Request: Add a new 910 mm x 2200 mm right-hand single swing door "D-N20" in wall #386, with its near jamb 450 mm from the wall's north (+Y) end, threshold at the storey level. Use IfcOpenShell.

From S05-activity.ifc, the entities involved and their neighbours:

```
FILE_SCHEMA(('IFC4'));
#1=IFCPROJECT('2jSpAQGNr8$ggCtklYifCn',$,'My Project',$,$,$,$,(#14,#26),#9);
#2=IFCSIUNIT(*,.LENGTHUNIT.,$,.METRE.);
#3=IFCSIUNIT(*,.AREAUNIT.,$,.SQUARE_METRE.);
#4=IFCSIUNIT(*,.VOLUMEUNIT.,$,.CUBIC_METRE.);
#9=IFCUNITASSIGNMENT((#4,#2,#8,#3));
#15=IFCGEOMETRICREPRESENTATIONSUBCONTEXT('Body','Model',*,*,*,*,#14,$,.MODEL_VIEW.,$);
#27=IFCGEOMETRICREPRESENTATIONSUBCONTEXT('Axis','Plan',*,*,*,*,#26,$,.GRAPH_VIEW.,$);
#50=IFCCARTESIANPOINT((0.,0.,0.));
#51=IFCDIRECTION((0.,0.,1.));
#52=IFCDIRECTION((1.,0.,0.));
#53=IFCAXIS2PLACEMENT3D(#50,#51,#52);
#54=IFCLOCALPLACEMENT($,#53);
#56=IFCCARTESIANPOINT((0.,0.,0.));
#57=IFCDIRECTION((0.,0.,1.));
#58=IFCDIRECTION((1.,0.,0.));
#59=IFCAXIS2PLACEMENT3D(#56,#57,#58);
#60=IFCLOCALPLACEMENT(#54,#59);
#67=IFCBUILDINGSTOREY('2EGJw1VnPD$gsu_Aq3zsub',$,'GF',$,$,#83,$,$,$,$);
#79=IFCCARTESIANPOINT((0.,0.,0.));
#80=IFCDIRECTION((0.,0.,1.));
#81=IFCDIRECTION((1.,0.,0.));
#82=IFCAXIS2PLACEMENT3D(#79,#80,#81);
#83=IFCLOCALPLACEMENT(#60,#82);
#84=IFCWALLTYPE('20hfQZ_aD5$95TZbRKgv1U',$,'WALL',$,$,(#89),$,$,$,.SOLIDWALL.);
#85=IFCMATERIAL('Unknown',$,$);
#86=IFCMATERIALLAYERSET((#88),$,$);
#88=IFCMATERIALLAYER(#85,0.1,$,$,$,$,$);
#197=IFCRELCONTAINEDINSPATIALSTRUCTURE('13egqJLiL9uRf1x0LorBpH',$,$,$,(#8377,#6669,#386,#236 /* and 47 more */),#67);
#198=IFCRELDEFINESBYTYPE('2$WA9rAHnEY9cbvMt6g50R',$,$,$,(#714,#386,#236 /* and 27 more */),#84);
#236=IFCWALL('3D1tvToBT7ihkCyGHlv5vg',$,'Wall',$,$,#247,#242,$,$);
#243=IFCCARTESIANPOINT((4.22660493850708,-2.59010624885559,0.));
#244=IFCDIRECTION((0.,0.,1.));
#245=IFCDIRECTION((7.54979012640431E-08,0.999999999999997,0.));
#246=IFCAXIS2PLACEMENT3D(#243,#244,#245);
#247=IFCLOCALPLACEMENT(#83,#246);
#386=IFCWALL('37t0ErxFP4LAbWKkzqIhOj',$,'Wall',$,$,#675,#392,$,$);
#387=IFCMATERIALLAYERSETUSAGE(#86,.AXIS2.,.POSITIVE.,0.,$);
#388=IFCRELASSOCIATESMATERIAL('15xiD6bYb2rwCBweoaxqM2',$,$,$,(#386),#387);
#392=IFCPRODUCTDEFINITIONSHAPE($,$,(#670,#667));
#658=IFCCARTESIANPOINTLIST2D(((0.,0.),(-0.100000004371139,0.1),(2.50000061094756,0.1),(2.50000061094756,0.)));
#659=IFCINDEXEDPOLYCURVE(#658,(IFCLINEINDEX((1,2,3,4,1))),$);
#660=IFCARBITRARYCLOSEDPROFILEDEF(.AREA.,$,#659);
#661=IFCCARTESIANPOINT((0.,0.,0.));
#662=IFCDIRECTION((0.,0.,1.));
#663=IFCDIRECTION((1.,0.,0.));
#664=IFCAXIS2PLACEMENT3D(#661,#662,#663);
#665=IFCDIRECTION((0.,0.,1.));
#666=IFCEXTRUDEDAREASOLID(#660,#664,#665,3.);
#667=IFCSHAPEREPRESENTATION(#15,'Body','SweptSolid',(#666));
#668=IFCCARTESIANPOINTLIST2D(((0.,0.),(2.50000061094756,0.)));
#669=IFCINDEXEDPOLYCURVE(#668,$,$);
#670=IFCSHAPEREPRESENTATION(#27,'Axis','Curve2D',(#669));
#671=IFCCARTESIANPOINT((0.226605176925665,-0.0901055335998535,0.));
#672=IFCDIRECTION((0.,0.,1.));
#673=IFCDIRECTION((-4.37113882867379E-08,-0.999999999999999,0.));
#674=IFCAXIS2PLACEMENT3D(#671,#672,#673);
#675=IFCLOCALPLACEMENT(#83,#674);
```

```python
import numpy as np
import ifcopenshell
import ifcopenshell.api.feature
import ifcopenshell.api.geometry
import ifcopenshell.api.root
import ifcopenshell.api.spatial
import ifcopenshell.geom
import ifcopenshell.util.element
import ifcopenshell.util.placement
import ifcopenshell.util.representation
import ifcopenshell.util.shape
import ifcopenshell.util.unit

model = ifcopenshell.open("S05-activity.ifc")
unit_scale = ifcopenshell.util.unit.calculate_unit_scale(model)
settings = ifcopenshell.geom.settings()


def volume(element):
    """Net volume in cubic metres, openings subtracted."""
    shape = ifcopenshell.geom.create_shape(settings, element)
    return ifcopenshell.util.shape.get_volume(shape.geometry)


wall = model.by_guid("37t0ErxFP4LAbWKkzqIhOj")
storey = ifcopenshell.util.element.get_container(wall, ifc_class="IfcBuildingStorey")
context = ifcopenshell.util.representation.get_context(model, "Model", "Body", "MODEL_VIEW")
before = volume(wall)

width, height, from_end, sill = 0.91, 2.2, 0.45, 0.0  # metres

# The wall runs along its own X axis, and the end named is its -X end.
wall_shape = ifcopenshell.geom.create_shape(settings, wall)
x, y, z = ifcopenshell.util.shape.get_vertices(wall_shape.geometry).T
start = x.min() + from_end
face, thickness = float(y.min()), float(y.max() - y.min())
wall_matrix = ifcopenshell.util.placement.get_local_placement(wall.ObjectPlacement)
level = ifcopenshell.util.placement.get_local_placement(storey.ObjectPlacement)[2, 3]


def in_wall(x, y):
    """Placement at x, y metres in the wall's axes, at sill height."""
    matrix = wall_matrix.copy()
    matrix[:, 3] = wall_matrix @ np.array([x / unit_scale, y / unit_scale, 0.0, 1.0])
    matrix[2, 3] = level + sill / unit_scale
    return matrix


# Opening: a box that overshoots both wall faces by 50 mm.
opening = ifcopenshell.api.root.create_entity(model, ifc_class="IfcOpeningElement", predefined_type="OPENING")
box = ifcopenshell.api.geometry.add_wall_representation(
    model, context=context, length=width, height=height, thickness=thickness + 0.1
)
ifcopenshell.api.geometry.assign_representation(model, product=opening, representation=box)
ifcopenshell.api.geometry.edit_object_placement(model, product=opening, matrix=in_wall(start, face - 0.05), is_si=False)
ifcopenshell.api.feature.add_feature(model, feature=opening, element=wall)

door = ifcopenshell.api.root.create_entity(model, ifc_class="IfcDoor", name="D-N20", predefined_type="DOOR")
door.OverallWidth, door.OverallHeight = width / unit_scale, height / unit_scale
door.OperationType = "SINGLE_SWING_RIGHT"
body = ifcopenshell.api.geometry.add_door_representation(
    model,
    context=context,
    overall_width=door.OverallWidth,
    overall_height=door.OverallHeight,
    operation_type="SINGLE_SWING_RIGHT",
    lining_properties={"LiningDepth": thickness / unit_scale, "ThresholdDepth": thickness / unit_scale},
)
ifcopenshell.api.geometry.assign_representation(model, product=door, representation=body)
ifcopenshell.api.spatial.assign_container(model, products=[door], relating_structure=storey)
ifcopenshell.api.feature.add_filling(model, opening=opening, element=door)

# The lining spans the wall, so the door starts at the wall face.
ifcopenshell.api.geometry.edit_object_placement(model, product=door, matrix=in_wall(start, face), is_si=False)

after = volume(wall)

print(f"wall volume {before:.3f} -> {after:.3f} m3")

model.write("S05-activity_updated.ifc")
```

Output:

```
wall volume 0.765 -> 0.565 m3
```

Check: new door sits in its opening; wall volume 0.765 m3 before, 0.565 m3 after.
